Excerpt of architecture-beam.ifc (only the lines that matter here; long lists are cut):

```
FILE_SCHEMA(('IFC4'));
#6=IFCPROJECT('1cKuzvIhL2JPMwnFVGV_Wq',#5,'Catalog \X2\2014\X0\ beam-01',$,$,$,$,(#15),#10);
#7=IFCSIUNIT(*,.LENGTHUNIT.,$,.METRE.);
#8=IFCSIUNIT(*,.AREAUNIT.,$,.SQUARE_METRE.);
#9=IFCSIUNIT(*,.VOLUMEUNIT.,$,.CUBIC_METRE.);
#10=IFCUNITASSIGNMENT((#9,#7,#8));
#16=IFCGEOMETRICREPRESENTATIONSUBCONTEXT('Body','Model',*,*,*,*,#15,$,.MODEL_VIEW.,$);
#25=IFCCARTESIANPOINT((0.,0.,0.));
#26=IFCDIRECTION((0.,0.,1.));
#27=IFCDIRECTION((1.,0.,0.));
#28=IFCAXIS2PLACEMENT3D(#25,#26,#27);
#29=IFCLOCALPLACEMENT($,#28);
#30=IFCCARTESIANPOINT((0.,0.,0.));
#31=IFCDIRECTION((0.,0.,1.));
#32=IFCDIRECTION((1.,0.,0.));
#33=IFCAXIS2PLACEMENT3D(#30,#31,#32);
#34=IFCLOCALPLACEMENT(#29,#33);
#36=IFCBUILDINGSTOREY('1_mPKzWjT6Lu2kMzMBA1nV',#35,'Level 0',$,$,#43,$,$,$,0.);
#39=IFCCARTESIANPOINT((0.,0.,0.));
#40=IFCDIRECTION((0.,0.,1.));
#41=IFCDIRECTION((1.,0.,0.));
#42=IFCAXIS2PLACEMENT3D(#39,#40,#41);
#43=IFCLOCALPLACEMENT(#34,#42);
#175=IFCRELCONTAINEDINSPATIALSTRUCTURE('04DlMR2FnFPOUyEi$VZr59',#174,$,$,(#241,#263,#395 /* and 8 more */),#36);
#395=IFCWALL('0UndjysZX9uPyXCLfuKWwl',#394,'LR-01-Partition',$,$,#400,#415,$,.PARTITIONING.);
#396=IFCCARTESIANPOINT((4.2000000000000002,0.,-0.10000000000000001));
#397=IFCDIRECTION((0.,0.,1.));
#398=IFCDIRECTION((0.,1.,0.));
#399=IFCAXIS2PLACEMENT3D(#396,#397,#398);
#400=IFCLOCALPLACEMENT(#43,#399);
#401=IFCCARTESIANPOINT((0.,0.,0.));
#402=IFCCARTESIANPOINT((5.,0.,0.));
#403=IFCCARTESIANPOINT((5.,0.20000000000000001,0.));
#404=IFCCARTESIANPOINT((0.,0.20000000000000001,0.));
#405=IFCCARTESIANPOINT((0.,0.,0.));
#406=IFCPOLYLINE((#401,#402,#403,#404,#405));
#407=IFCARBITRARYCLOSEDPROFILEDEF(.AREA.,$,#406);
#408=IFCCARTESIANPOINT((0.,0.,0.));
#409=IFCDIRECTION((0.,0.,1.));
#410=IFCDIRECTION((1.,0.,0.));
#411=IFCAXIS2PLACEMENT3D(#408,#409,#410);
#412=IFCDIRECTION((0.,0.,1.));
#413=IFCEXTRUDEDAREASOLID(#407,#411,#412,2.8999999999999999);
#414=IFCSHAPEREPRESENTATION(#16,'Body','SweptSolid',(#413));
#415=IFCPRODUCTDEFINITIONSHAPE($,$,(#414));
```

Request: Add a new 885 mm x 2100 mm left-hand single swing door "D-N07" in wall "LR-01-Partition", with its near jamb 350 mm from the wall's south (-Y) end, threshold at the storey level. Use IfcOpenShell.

```python
import numpy as np
import ifcopenshell
import ifcopenshell.api.feature
import ifcopenshell.api.geometry
import ifcopenshell.api.root
import ifcopenshell.api.spatial
import ifcopenshell.geom
import ifcopenshell.util.element
import ifcopenshell.util.placement
import ifcopenshell.util.representation
import ifcopenshell.util.shape
import ifcopenshell.util.unit

model = ifcopenshell.open("architecture-beam.ifc")
unit_scale = ifcopenshell.util.unit.calculate_unit_scale(model)
settings = ifcopenshell.geom.settings()


def volume(element):
    """Net volume in cubic metres, openings subtracted."""
    shape = ifcopenshell.geom.create_shape(settings, element)
    return ifcopenshell.util.shape.get_volume(shape.geometry)


wall = model.by_guid("0UndjysZX9uPyXCLfuKWwl")
storey = ifcopenshell.util.element.get_container(wall, ifc_class="IfcBuildingStorey")
context = ifcopenshell.util.representation.get_context(model, "Model", "Body", "MODEL_VIEW")
before = volume(wall)

width, height, from_end, sill = 0.885, 2.1, 0.35, 0.0  # metres

# The wall runs along its own X axis, and the end named is its -X end.
wall_shape = ifcopenshell.geom.create_shape(settings, wall)
x, y, z = ifcopenshell.util.shape.get_vertices(wall_shape.geometry).T
start = x.min() + from_end
face, thickness = float(y.min()), float(y.max() - y.min())
wall_matrix = ifcopenshell.util.placement.get_local_placement(wall.ObjectPlacement)
level = ifcopenshell.util.placement.get_local_placement(storey.ObjectPlacement)[2, 3]


def in_wall(x, y):
    """Placement at x, y metres in the wall's axes, at sill height."""
    matrix = wall_matrix.copy()
    matrix[:, 3] = wall_matrix @ np.array([x / unit_scale, y / unit_scale, 0.0, 1.0])
    matrix[2, 3] = level + sill / unit_scale
    return matrix


# Opening: a box that overshoots both wall faces by 50 mm.
opening = ifcopenshell.api.root.create_entity(model, ifc_class="IfcOpeningElement", predefined_type="OPENING")
box = ifcopenshell.api.geometry.add_wall_representation(
    model, context=context, length=width, height=height, thickness=thickness + 0.1
)
ifcopenshell.api.geometry.assign_representation(model, product=opening, representation=box)
ifcopenshell.api.geometry.edit_object_placement(model, product=opening, matrix=in_wall(start, face - 0.05), is_si=False)
ifcopenshell.api.feature.add_feature(model, feature=opening, element=wall)

door = ifcopenshell.api.root.create_entity(model, ifc_class="IfcDoor", name="D-N07", predefined_type="DOOR")
door.OverallWidth, door.OverallHeight = width / unit_scale, height / unit_scale
door.OperationType = "SINGLE_SWING_LEFT"
body = ifcopenshell.api.geometry.add_door_representation(
    model,
    context=context,
    overall_width=door.OverallWidth,
    overall_height=door.OverallHeight,
    operation_type="SINGLE_SWING_LEFT",
    lining_properties={"LiningDepth": thickness / unit_scale, "ThresholdDepth": thickness / unit_scale},
)
ifcopenshell.api.geometry.assign_representation(model, product=door, representation=body)
ifcopenshell.api.spatial.assign_container(model, products=[door], relating_structure=storey)
ifcopenshell.api.feature.add_filling(model, opening=opening, element=door)

# The lining spans the wall, so the door starts at the wall face.
ifcopenshell.api.geometry.edit_object_placement(model, product=door, matrix=in_wall(start, face), is_si=False)

after = volume(wall)

print(f"wall volume {before:.3f} -> {after:.3f} m3")

model.write("architecture-beam_edited.ifc")
```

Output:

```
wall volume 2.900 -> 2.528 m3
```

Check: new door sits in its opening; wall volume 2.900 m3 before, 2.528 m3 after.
